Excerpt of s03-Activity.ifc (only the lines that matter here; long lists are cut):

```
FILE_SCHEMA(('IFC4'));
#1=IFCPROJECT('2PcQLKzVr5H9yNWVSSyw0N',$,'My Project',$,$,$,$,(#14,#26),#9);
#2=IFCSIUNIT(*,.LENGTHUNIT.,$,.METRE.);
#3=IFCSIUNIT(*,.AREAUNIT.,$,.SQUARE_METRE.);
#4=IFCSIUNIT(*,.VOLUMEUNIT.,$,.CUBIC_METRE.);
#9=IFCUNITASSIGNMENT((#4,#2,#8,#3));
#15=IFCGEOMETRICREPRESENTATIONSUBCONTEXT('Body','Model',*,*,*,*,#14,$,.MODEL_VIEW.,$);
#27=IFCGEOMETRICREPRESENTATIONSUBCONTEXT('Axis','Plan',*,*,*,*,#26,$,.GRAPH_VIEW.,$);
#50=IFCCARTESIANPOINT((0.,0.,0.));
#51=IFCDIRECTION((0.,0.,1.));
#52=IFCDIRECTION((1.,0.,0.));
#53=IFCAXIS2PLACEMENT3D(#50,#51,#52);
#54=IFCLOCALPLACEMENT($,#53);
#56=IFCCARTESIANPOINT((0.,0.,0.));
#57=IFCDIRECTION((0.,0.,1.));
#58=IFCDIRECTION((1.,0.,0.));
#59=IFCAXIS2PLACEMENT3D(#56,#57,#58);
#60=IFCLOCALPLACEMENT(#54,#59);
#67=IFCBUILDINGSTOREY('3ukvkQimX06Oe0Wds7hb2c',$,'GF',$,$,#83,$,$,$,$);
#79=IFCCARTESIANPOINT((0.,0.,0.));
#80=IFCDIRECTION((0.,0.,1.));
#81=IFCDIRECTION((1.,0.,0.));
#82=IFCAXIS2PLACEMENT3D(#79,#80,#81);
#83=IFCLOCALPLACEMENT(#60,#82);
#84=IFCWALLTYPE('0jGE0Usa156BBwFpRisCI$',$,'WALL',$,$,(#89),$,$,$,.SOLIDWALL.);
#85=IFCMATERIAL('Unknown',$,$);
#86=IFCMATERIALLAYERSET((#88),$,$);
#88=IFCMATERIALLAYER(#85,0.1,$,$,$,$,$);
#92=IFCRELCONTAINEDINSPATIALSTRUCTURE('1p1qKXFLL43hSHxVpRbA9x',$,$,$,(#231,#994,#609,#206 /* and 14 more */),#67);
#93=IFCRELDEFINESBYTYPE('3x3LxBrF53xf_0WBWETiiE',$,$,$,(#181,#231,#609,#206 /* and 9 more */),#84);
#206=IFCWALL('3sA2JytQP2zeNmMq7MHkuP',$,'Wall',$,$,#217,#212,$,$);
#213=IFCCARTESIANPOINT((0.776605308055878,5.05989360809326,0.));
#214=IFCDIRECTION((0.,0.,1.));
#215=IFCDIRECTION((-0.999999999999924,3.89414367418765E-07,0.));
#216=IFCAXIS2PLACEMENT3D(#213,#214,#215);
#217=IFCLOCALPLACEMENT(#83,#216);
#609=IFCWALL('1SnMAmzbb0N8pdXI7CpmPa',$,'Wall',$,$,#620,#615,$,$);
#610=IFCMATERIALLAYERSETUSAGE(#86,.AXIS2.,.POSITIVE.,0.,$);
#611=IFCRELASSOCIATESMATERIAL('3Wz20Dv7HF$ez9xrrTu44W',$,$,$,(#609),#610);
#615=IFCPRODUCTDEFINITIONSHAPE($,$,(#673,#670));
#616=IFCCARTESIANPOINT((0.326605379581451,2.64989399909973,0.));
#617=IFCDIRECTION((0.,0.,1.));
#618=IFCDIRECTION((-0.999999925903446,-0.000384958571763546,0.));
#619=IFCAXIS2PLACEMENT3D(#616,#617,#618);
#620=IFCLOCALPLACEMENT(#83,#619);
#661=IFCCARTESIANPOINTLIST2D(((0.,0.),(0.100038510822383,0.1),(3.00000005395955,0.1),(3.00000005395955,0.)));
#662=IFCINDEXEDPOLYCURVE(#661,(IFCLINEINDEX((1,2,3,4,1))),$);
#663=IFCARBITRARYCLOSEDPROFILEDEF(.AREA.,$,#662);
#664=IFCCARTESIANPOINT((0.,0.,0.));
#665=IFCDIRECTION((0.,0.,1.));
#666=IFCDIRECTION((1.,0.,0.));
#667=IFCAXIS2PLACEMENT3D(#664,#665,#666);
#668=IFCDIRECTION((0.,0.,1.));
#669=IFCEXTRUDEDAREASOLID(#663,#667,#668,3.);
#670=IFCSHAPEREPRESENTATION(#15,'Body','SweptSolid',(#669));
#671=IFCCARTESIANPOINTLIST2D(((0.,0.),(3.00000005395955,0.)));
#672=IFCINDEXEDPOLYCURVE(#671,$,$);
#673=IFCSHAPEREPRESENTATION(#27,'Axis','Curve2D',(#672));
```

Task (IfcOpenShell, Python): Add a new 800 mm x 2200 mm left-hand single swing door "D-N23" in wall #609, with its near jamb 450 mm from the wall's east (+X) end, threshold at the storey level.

```python
import numpy as np
import ifcopenshell
import ifcopenshell.api.feature
import ifcopenshell.api.geometry
import ifcopenshell.api.root
import ifcopenshell.api.spatial
import ifcopenshell.geom
import ifcopenshell.util.element
import ifcopenshell.util.placement
import ifcopenshell.util.representation
import ifcopenshell.util.shape
import ifcopenshell.util.unit

model = ifcopenshell.open("s03-Activity.ifc")
unit_scale = ifcopenshell.util.unit.calculate_unit_scale(model)
settings = ifcopenshell.geom.settings()


def volume(element):
    """Net volume in cubic metres, openings subtracted."""
    shape = ifcopenshell.geom.create_shape(settings, element)
    return ifcopenshell.util.shape.get_volume(shape.geometry)


wall = model.by_guid("1SnMAmzbb0N8pdXI7CpmPa")
storey = ifcopenshell.util.element.get_container(wall, ifc_class="IfcBuildingStorey")
context = ifcopenshell.util.representation.get_context(model, "Model", "Body", "MODEL_VIEW")
before = volume(wall)

width, height, from_end, sill = 0.8, 2.2, 0.45, 0.0  # metres

# The wall runs along its own X axis, and the end named is its -X end.
wall_shape = ifcopenshell.geom.create_shape(settings, wall)
x, y, z = ifcopenshell.util.shape.get_vertices(wall_shape.geometry).T
start = x.min() + from_end
face, thickness = float(y.min()), float(y.max() - y.min())
wall_matrix = ifcopenshell.util.placement.get_local_placement(wall.ObjectPlacement)
level = ifcopenshell.util.placement.get_local_placement(storey.ObjectPlacement)[2, 3]


def in_wall(x, y):
    """Placement at x, y metres in the wall's axes, at sill height."""
    matrix = wall_matrix.copy()
    matrix[:, 3] = wall_matrix @ np.array([x / unit_scale, y / unit_scale, 0.0, 1.0])
    matrix[2, 3] = level + sill / unit_scale
    return matrix


# Opening: a box that overshoots both wall faces by 50 mm.
opening = ifcopenshell.api.root.create_entity(model, ifc_class="IfcOpeningElement", predefined_type="OPENING")
box = ifcopenshell.api.geometry.add_wall_representation(
    model, context=context, length=width, height=height, thickness=thickness + 0.1
)
ifcopenshell.api.geometry.assign_representation(model, product=opening, representation=box)
ifcopenshell.api.geometry.edit_object_placement(model, product=opening, matrix=in_wall(start, face - 0.05), is_si=False)
ifcopenshell.api.feature.add_feature(model, feature=opening, element=wall)

door = ifcopenshell.api.root.create_entity(model, ifc_class="IfcDoor", name="D-N23", predefined_type="DOOR")
door.OverallWidth, door.OverallHeight = width / unit_scale, height / unit_scale
door.OperationType = "SINGLE_SWING_LEFT"
body = ifcopenshell.api.geometry.add_door_representation(
    model,
    context=context,
    overall_width=door.OverallWidth,
    overall_height=door.OverallHeight,
    operation_type="SINGLE_SWING_LEFT",
    lining_properties={"LiningDepth": thickness / unit_scale, "ThresholdDepth": thickness / unit_scale},
)
ifcopenshell.api.geometry.assign_representation(model, product=door, representation=body)
ifcopenshell.api.spatial.assign_container(model, products=[door], relating_structure=storey)
ifcopenshell.api.feature.add_filling(model, opening=opening, element=door)

# The lining spans the wall, so the door starts at the wall face.
ifcopenshell.api.geometry.edit_object_placement(model, product=door, matrix=in_wall(start, face), is_si=False)

after = volume(wall)

print(f"wall volume {before:.3f} -> {after:.3f} m3")

model.write("s03-Activity_edited.ifc")
```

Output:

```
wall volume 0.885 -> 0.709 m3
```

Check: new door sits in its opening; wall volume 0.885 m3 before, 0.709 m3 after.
